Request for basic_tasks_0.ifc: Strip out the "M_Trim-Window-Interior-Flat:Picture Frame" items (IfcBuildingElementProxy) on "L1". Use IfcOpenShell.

First a look at what the model holds.

```python
import ifcopenshell
import ifcopenshell.util.element

model = ifcopenshell.open("basic_tasks_0.ifc")
print(model.schema)
storey = next(s for s in model.by_type("IfcBuildingStorey") if s.Name == "L1")
proxies = [e for e in ifcopenshell.util.element.get_decomposition(storey) if e.is_a("IfcBuildingElementProxy")]
seen = {}
for e in proxies:
    element_type = ifcopenshell.util.element.get_type(e)
    name = element_type.Name if element_type not in (None, e) else None
    seen[name] = seen.get(name, 0) + 1
for name, count in sorted(seen.items(), key=str):
    print(count, "x", name)
```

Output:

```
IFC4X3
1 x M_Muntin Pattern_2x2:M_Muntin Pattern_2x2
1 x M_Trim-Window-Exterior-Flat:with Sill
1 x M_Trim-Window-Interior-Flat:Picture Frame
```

```python
import ifcopenshell
import ifcopenshell.api.root
import ifcopenshell.util.element

model = ifcopenshell.open("basic_tasks_0.ifc")

storey = next(s for s in model.by_type("IfcBuildingStorey") if s.Name == "L1")
proxies = [e for e in ifcopenshell.util.element.get_decomposition(storey) if e.is_a("IfcBuildingElementProxy")]
targets = [e for e in proxies if (t := ifcopenshell.util.element.get_type(e)) not in (None, e) and t.Name == "M_Trim-Window-Interior-Flat:Picture Frame"]

for e in targets:
    ifcopenshell.api.root.remove_product(model, product=e)
print(len(targets), "removed")

model.write("basic_tasks_0_rev.ifc")
```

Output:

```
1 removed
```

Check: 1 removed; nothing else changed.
